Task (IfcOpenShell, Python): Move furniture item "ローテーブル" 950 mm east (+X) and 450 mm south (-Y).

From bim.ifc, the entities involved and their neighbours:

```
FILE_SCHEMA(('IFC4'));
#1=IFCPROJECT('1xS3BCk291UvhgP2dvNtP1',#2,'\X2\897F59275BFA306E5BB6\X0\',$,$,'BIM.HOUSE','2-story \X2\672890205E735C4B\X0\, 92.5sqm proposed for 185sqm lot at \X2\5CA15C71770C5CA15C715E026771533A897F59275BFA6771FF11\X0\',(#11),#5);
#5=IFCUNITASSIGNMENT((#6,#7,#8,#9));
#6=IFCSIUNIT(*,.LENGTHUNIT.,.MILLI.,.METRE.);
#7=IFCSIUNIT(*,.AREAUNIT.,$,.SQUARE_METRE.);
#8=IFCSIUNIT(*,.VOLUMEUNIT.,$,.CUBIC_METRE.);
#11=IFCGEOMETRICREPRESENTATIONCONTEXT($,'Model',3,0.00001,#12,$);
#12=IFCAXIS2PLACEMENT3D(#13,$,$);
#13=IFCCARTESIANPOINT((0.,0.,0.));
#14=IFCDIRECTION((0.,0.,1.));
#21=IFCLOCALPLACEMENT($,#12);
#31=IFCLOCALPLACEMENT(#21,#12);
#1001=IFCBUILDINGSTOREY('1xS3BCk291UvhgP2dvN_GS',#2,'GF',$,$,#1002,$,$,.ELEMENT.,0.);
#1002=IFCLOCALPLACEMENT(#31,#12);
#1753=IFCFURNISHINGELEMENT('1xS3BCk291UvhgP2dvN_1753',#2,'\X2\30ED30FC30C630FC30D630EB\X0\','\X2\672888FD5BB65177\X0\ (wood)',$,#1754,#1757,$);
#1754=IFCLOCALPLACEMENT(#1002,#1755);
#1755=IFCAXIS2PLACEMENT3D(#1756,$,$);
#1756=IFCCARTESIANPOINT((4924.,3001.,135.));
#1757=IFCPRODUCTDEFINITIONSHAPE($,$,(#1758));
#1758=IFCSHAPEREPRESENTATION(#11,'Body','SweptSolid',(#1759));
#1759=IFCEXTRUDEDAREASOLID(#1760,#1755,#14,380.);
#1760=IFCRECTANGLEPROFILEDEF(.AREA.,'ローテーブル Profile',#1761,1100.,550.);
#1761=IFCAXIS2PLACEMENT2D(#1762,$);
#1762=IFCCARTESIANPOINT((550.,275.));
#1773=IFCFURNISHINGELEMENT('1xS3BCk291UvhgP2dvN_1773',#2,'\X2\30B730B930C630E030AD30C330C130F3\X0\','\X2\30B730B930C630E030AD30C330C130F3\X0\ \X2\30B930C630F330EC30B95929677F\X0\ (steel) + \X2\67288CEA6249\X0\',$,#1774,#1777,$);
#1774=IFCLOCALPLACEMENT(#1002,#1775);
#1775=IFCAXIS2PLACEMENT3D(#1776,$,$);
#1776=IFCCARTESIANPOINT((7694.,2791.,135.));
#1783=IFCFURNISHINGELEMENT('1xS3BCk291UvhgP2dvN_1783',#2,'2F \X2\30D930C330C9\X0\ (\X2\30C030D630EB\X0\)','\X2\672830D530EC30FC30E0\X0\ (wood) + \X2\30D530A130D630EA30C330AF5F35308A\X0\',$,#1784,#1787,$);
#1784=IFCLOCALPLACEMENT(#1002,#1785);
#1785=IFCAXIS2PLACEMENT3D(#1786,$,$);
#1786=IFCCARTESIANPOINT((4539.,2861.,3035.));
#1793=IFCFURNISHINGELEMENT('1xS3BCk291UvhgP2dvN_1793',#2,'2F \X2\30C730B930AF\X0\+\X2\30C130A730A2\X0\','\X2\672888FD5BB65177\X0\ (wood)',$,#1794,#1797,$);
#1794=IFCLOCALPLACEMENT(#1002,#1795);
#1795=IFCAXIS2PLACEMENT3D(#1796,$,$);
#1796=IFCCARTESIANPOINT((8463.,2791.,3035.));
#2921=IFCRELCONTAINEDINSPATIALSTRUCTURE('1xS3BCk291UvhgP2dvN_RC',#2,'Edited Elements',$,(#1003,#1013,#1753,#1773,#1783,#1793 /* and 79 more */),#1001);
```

```python
import ifcopenshell
import ifcopenshell.api.geometry
import ifcopenshell.util.placement
import ifcopenshell.util.unit

model = ifcopenshell.open("bim.ifc")
unit_scale = ifcopenshell.util.unit.calculate_unit_scale(model)

item = model.by_guid("1xS3BCk291UvhgP2dvN_1753")
matrix = ifcopenshell.util.placement.get_local_placement(item.ObjectPlacement)
matrix[0, 3] += 0.95 / unit_scale
matrix[1, 3] -= 0.45 / unit_scale
ifcopenshell.api.geometry.edit_object_placement(model, product=item, matrix=matrix, is_si=False)

print(ifcopenshell.util.placement.get_local_placement(item.ObjectPlacement).round(3) + 0.0)

model.write("bim_v2.ifc")
```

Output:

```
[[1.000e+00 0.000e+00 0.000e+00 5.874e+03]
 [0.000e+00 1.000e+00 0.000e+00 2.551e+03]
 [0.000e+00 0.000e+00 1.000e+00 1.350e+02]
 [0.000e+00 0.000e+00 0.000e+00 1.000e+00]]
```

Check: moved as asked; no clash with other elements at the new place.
